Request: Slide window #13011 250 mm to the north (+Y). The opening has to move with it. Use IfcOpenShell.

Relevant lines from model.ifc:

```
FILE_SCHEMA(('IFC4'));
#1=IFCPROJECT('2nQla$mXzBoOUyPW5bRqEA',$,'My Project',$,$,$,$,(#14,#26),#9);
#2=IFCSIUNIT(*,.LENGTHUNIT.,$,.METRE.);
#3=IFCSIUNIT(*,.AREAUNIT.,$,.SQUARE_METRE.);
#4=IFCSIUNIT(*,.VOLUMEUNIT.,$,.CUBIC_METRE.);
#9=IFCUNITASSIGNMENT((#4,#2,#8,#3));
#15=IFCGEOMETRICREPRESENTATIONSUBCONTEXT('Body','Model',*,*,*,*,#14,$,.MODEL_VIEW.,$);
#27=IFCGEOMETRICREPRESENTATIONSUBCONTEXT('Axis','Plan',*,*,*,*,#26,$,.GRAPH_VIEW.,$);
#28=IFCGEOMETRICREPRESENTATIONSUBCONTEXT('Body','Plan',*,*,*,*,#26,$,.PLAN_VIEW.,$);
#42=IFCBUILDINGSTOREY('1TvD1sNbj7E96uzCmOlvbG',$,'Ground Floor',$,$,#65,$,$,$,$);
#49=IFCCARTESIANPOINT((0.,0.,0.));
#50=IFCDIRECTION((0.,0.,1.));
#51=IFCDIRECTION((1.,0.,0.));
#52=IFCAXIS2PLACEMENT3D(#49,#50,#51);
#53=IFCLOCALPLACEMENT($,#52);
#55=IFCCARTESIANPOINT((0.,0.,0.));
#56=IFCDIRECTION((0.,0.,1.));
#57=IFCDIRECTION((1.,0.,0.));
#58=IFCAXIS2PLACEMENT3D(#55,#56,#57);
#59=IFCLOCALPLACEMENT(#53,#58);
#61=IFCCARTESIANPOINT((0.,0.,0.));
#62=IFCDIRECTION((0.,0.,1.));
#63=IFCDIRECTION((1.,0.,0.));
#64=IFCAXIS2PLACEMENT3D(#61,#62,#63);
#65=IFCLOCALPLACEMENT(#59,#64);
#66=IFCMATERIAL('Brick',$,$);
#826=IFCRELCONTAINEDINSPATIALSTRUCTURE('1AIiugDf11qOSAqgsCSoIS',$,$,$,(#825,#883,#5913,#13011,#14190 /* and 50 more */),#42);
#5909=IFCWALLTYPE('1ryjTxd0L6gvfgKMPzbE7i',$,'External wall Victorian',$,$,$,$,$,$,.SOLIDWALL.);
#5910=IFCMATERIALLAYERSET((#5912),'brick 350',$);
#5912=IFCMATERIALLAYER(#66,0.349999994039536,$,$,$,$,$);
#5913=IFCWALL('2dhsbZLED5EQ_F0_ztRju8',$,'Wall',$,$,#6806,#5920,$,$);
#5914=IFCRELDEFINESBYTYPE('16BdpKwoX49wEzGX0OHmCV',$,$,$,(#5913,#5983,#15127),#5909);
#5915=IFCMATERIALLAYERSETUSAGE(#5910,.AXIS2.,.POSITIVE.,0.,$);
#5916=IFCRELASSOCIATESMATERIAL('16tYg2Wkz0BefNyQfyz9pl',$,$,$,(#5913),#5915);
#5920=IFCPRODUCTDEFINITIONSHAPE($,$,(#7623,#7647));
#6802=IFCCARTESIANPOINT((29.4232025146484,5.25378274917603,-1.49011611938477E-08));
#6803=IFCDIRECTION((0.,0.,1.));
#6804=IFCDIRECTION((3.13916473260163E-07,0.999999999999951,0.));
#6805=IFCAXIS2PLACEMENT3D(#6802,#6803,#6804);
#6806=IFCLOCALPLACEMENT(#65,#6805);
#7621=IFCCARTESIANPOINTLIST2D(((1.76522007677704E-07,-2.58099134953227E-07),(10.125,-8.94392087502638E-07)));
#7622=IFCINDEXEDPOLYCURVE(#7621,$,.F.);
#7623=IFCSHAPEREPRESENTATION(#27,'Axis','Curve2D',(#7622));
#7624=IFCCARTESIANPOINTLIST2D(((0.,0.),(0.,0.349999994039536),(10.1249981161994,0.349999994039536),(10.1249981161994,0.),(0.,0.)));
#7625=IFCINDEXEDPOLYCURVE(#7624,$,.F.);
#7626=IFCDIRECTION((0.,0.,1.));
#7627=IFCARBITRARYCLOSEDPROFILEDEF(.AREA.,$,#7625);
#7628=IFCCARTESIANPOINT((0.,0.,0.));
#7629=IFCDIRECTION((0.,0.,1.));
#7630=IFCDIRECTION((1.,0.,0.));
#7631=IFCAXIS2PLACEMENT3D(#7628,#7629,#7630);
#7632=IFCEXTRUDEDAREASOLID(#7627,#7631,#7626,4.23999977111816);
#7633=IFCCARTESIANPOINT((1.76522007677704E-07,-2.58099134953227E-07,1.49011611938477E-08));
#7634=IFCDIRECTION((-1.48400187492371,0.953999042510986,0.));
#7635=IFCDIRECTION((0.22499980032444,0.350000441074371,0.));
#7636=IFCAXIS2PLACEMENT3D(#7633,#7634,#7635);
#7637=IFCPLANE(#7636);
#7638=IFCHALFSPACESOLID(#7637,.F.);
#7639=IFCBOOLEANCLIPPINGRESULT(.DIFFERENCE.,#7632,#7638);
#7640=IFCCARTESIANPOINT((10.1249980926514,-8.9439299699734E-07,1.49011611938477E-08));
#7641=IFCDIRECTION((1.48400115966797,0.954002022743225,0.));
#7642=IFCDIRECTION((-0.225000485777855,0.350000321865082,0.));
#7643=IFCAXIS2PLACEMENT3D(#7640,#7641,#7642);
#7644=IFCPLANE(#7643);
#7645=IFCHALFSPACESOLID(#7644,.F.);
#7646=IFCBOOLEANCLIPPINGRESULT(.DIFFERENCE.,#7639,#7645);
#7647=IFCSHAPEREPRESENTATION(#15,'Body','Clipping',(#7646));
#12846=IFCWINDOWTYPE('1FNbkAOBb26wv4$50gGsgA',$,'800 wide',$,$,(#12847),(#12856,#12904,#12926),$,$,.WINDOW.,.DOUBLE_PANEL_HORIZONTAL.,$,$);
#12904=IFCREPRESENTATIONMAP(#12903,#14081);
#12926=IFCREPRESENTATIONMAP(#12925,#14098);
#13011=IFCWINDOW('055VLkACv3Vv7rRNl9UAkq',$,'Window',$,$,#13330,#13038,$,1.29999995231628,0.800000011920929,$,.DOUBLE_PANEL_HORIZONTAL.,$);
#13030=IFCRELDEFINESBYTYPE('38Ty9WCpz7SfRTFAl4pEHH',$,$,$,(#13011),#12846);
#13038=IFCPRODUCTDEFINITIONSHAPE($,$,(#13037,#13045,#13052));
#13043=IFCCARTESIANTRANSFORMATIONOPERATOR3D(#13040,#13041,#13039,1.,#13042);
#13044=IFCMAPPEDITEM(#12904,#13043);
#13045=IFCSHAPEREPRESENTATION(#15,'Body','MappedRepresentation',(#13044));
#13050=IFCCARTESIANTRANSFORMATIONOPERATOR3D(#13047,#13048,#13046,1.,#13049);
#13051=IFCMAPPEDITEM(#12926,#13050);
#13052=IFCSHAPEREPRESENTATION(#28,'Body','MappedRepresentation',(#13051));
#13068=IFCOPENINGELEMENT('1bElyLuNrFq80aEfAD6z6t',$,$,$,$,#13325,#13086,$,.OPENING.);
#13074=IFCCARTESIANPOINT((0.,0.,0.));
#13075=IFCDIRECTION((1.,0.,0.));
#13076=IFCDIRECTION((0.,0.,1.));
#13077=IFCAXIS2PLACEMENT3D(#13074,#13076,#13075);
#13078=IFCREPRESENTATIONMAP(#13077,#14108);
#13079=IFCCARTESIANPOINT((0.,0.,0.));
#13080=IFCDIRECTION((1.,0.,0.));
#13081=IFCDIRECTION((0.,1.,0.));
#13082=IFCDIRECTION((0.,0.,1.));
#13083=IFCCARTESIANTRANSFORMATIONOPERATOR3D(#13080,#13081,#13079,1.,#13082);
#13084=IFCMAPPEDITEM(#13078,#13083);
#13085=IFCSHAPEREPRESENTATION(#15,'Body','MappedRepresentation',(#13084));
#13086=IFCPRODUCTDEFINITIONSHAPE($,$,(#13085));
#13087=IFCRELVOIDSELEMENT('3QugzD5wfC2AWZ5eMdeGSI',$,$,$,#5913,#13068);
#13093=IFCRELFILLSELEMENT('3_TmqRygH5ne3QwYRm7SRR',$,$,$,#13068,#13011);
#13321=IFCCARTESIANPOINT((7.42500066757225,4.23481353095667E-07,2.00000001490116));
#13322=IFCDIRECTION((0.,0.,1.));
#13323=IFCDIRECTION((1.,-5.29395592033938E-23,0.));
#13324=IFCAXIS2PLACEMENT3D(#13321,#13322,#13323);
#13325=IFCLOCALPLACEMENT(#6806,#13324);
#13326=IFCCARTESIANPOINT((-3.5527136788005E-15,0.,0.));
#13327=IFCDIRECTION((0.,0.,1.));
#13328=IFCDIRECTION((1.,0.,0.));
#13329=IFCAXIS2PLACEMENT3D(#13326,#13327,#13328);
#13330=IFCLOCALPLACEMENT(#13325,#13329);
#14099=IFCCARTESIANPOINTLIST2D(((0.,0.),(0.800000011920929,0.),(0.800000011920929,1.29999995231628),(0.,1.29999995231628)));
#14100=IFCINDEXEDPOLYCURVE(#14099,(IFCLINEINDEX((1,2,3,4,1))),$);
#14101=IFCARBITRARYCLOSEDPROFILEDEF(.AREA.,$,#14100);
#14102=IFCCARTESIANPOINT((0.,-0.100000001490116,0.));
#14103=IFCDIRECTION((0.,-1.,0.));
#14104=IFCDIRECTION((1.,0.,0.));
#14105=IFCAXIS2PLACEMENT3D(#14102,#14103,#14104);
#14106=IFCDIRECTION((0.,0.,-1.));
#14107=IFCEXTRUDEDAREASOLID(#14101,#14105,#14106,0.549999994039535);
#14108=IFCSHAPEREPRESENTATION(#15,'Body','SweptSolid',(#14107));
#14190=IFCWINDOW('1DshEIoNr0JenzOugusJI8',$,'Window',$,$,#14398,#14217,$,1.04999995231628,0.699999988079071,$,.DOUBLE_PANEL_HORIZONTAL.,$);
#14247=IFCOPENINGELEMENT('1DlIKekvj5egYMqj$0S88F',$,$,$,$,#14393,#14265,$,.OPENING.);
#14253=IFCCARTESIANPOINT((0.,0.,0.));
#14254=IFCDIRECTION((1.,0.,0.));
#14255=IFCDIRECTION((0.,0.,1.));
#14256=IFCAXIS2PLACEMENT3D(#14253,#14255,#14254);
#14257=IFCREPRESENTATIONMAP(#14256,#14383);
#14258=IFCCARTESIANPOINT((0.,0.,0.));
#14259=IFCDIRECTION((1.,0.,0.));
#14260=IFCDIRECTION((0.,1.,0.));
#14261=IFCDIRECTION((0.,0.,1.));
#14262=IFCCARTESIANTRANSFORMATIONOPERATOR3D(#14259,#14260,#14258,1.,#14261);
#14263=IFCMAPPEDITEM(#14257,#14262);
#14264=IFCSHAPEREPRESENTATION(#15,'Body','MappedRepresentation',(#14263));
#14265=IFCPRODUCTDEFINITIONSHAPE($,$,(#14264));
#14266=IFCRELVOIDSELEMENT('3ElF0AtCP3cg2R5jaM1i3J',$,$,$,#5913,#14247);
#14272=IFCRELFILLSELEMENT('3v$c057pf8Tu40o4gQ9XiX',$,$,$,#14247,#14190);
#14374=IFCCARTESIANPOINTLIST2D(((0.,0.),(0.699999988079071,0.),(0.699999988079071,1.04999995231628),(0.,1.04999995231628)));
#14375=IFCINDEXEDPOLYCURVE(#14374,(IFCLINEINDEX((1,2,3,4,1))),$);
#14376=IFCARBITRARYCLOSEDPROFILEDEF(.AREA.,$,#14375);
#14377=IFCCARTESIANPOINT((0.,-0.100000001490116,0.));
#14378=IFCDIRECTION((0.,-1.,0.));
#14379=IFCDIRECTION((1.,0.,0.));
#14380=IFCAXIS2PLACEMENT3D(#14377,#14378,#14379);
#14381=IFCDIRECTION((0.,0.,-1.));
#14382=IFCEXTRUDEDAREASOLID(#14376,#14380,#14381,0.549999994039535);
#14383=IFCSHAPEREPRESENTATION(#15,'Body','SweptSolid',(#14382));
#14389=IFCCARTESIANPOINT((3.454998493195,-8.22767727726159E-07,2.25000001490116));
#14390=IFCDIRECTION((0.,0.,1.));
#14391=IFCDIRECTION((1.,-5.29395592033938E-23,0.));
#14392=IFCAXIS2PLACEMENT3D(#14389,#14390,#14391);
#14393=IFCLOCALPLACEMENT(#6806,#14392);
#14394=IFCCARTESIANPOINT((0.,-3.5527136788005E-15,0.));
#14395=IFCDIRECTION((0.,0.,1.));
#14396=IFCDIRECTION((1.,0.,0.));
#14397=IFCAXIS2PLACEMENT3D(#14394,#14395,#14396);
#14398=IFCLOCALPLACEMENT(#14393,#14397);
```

```python
import ifcopenshell
import ifcopenshell.api.geometry
import ifcopenshell.util.placement
import ifcopenshell.util.unit

model = ifcopenshell.open("model.ifc")
unit_scale = ifcopenshell.util.unit.calculate_unit_scale(model)

window = model.by_guid("055VLkACv3Vv7rRNl9UAkq")
opening = window.FillsVoids[0].RelatingOpeningElement
wall = opening.VoidsElements[0].RelatingBuildingElement

wall_matrix = ifcopenshell.util.placement.get_local_placement(wall.ObjectPlacement)
shift = wall_matrix[:3, 0] * 0.25 / unit_scale
before = ifcopenshell.util.placement.get_local_placement(window.ObjectPlacement)[:3, 3].copy()

# The window is placed relative to its opening, so it follows when the opening moves.
matrix = ifcopenshell.util.placement.get_local_placement(opening.ObjectPlacement)
matrix[:3, 3] += shift
ifcopenshell.api.geometry.edit_object_placement(
    model, product=opening, matrix=matrix, is_si=False, should_transform_children=True
)

after = ifcopenshell.util.placement.get_local_placement(window.ObjectPlacement)[:3, 3]
print("window moved by", (after - before).round(3) + 0.0)

model.write("model_v2.ifc")
```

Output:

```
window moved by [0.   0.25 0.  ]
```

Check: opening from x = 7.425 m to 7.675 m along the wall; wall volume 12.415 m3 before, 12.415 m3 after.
